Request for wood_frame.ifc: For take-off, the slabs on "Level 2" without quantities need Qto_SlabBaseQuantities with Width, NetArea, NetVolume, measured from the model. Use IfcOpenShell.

First a look at what the model holds.

```python
import ifcopenshell
import ifcopenshell.util.element
import ifcopenshell.util.unit

model = ifcopenshell.open("wood_frame.ifc")
print(model.schema)
for unit_type in ("LENGTHUNIT", "AREAUNIT", "VOLUMEUNIT"):
    print(unit_type, ifcopenshell.util.unit.calculate_unit_scale(model, unit_type))
storey = next(s for s in model.by_type("IfcBuildingStorey") if s.Name == "Level 2")
slabs = [e for e in ifcopenshell.util.element.get_decomposition(storey) if e.is_a("IfcSlab")]
for e in sorted(slabs, key=lambda e: e.id()):
    print(e.id(), e.is_a(), e.Name, list(ifcopenshell.util.element.get_psets(e, qtos_only=True)), sep=" | ")
```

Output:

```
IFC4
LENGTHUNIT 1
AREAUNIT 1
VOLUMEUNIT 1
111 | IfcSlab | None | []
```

```python
import ifcopenshell
import ifcopenshell.api.pset
import ifcopenshell.geom
import ifcopenshell.util.element
import ifcopenshell.util.shape
import ifcopenshell.util.unit

model = ifcopenshell.open("wood_frame.ifc")
unit_scale = ifcopenshell.util.unit.calculate_unit_scale(model)
area_scale = ifcopenshell.util.unit.calculate_unit_scale(model, "AREAUNIT")
volume_scale = ifcopenshell.util.unit.calculate_unit_scale(model, "VOLUMEUNIT")
settings = ifcopenshell.geom.settings()

storey = next(s for s in model.by_type("IfcBuildingStorey") if s.Name == "Level 2")
slabs = [e for e in ifcopenshell.util.element.get_decomposition(storey) if e.is_a("IfcSlab")]

for e in sorted(slabs, key=lambda e: e.id()):
    if ifcopenshell.util.element.get_psets(e, qtos_only=True, should_inherit=False):
        continue
    # Geometry comes back in metres, in the element's own axes.
    shape = ifcopenshell.geom.create_shape(settings, e)
    values = {
        "Width": ifcopenshell.util.shape.get_z(shape.geometry) / unit_scale,
        "NetArea": ifcopenshell.util.shape.get_footprint_area(shape.geometry) / area_scale,
        "NetVolume": ifcopenshell.util.shape.get_volume(shape.geometry) / volume_scale,
    }
    qto = ifcopenshell.api.pset.add_qto(model, product=e, name="Qto_SlabBaseQuantities")
    ifcopenshell.api.pset.edit_qto(model, qto=qto, properties=values)
    print(e.id(), {k: round(v, 3) for k, v in values.items()})

model.write("wood_frame_rev.ifc")
```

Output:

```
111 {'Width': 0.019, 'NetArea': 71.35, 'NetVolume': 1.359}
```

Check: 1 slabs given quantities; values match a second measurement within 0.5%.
